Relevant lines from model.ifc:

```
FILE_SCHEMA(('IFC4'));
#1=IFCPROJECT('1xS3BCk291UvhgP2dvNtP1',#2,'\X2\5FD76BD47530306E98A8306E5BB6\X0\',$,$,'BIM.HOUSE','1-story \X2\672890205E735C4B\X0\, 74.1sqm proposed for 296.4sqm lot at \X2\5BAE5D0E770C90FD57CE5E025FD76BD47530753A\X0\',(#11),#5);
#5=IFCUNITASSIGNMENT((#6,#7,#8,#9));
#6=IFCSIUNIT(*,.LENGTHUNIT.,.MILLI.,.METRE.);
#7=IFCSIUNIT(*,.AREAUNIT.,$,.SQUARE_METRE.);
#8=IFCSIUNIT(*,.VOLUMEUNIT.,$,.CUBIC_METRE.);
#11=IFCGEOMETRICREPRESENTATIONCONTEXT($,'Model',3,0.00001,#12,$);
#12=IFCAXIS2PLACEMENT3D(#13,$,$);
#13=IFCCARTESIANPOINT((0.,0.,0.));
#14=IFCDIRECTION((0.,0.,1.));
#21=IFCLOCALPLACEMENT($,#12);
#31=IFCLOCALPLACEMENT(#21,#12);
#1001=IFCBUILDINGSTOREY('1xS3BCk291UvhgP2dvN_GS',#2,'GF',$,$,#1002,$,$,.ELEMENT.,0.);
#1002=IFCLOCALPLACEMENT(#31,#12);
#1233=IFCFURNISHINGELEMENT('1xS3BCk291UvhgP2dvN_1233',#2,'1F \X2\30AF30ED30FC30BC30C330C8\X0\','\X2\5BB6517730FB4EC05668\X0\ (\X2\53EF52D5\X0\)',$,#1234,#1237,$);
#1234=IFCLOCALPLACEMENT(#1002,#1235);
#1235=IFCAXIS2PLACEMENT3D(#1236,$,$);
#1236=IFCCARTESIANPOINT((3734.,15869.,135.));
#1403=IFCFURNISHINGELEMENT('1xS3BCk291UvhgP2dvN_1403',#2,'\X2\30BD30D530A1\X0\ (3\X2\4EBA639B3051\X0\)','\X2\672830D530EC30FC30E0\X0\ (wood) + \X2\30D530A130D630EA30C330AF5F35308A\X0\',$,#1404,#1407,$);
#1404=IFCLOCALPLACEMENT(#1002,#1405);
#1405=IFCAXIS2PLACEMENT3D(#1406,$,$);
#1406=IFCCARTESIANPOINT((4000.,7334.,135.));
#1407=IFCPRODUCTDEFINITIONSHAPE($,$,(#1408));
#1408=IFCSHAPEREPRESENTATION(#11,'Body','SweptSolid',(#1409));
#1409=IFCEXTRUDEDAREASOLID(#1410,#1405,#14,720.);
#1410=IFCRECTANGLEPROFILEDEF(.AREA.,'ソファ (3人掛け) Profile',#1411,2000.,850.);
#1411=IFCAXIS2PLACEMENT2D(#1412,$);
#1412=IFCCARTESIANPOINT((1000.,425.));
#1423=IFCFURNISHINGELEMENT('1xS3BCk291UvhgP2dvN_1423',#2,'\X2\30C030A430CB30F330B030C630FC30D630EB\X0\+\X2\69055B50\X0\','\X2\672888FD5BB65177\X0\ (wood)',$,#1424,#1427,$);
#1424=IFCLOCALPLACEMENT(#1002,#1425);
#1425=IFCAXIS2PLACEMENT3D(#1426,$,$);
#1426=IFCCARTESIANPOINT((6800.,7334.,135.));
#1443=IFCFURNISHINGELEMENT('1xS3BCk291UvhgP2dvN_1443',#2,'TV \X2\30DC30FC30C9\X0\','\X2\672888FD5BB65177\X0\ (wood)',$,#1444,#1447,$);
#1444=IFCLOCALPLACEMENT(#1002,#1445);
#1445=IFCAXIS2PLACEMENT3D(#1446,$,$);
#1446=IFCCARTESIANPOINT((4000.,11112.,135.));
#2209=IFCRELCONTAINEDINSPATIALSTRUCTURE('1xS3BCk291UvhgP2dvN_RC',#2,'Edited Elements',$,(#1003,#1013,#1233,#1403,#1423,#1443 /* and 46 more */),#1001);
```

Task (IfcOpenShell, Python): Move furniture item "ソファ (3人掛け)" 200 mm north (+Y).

```python
import ifcopenshell
import ifcopenshell.api.geometry
import ifcopenshell.util.placement
import ifcopenshell.util.unit

model = ifcopenshell.open("model.ifc")
unit_scale = ifcopenshell.util.unit.calculate_unit_scale(model)

item = model.by_guid("1xS3BCk291UvhgP2dvN_1403")
matrix = ifcopenshell.util.placement.get_local_placement(item.ObjectPlacement)
matrix[1, 3] += 0.2 / unit_scale
ifcopenshell.api.geometry.edit_object_placement(model, product=item, matrix=matrix, is_si=False)

print(ifcopenshell.util.placement.get_local_placement(item.ObjectPlacement).round(3) + 0.0)

model.write("model_rev.ifc")
```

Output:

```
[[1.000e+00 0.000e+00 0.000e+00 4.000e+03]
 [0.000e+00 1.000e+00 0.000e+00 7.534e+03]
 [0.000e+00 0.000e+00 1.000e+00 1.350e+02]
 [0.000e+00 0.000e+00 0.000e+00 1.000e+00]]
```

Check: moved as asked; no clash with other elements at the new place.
